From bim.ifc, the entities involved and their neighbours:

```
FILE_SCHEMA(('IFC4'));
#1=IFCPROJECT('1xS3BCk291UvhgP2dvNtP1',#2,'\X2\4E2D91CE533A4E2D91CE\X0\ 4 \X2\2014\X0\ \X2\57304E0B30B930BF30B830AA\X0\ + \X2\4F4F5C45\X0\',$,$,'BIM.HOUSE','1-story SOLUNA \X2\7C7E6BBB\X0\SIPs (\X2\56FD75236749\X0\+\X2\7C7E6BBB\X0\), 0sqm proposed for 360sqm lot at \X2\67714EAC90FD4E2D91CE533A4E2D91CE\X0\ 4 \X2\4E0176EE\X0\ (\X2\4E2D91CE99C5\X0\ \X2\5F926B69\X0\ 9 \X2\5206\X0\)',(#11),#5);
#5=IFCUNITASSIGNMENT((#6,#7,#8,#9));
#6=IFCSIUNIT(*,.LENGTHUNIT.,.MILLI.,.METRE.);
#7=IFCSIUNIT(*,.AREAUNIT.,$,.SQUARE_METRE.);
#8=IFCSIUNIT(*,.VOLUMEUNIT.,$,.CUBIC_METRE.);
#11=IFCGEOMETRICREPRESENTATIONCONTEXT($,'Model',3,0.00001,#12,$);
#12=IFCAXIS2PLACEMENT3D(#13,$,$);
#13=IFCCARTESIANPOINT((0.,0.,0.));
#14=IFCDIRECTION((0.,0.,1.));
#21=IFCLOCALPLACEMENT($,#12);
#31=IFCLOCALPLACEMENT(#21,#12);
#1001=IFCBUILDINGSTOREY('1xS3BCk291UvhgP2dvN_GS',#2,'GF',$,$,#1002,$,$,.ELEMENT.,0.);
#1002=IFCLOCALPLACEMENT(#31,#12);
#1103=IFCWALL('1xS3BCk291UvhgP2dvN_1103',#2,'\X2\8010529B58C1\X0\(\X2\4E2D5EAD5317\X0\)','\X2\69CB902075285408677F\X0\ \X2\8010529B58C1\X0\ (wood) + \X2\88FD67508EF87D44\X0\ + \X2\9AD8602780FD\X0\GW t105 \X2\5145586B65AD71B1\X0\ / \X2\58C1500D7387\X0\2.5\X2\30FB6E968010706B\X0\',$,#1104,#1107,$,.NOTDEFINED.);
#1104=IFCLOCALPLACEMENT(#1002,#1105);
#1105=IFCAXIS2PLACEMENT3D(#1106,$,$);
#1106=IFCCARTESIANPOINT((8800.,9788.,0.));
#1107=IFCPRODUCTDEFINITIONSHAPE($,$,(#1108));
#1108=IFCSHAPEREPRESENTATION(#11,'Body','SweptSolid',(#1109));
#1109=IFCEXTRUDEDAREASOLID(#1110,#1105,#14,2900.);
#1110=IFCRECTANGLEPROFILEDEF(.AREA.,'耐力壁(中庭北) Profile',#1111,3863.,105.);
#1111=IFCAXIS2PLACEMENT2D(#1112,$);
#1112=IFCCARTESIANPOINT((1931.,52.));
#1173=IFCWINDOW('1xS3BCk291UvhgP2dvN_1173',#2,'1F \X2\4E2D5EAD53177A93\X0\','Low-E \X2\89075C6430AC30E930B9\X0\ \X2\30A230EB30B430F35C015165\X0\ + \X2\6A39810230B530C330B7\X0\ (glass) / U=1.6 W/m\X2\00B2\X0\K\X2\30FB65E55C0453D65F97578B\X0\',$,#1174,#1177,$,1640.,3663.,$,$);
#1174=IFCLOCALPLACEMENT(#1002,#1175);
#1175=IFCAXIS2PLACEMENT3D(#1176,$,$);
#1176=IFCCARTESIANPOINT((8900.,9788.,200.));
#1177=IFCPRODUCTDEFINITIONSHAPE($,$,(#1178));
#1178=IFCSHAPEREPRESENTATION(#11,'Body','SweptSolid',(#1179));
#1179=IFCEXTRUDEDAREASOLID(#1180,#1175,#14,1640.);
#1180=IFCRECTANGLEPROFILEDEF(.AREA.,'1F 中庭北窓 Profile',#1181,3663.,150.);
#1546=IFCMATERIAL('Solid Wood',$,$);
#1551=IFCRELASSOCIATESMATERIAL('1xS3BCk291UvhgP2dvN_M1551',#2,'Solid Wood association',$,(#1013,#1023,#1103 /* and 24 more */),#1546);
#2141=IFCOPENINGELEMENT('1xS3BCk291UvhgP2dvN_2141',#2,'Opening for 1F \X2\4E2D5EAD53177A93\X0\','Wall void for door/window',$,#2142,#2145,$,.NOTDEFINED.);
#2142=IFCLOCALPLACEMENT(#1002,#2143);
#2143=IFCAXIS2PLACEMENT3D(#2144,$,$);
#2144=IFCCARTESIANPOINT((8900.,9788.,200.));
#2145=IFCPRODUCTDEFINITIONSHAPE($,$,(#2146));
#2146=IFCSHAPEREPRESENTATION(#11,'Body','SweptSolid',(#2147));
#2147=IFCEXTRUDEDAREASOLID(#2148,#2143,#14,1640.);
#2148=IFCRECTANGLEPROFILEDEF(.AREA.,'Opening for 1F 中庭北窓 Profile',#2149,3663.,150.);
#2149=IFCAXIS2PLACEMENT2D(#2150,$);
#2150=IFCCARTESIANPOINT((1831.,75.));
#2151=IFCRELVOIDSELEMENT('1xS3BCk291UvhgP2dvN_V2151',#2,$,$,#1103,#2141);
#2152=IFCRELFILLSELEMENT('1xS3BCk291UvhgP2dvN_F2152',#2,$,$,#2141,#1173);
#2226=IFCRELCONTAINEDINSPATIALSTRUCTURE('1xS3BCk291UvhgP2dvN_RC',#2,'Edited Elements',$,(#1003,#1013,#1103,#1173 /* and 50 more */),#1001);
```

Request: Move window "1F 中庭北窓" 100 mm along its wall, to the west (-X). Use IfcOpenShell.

```python
import ifcopenshell
import ifcopenshell.api.geometry
import ifcopenshell.util.placement

model = ifcopenshell.open("bim.ifc")

window = model.by_guid("1xS3BCk291UvhgP2dvN_1173")
opening = window.FillsVoids[0].RelatingOpeningElement
wall = opening.VoidsElements[0].RelatingBuildingElement

wall_matrix = ifcopenshell.util.placement.get_local_placement(wall.ObjectPlacement)
shift = wall_matrix[:3, 0] * -100.0
before = ifcopenshell.util.placement.get_local_placement(window.ObjectPlacement)[:3, 3].copy()

# The window is not placed relative to its opening, so move both.
for product in (opening, window):
    matrix = ifcopenshell.util.placement.get_local_placement(product.ObjectPlacement)
    matrix[:3, 3] += shift
    ifcopenshell.api.geometry.edit_object_placement(model, product=product, matrix=matrix, is_si=False)

after = ifcopenshell.util.placement.get_local_placement(window.ObjectPlacement)[:3, 3]
print("window moved by", (after - before).round(3) + 0.0)

model.write("bim-out.ifc")
```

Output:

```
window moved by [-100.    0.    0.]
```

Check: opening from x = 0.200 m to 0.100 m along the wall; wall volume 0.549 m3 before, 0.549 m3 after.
